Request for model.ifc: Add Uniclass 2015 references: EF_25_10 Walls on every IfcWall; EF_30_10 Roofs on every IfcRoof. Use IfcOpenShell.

First a look at what the model holds.

```python
import ifcopenshell

model = ifcopenshell.open("model.ifc")
print(model.schema)
print("classifications:", [c.Name for c in model.by_type("IfcClassification")])
for ifc_class in ("IfcDoor", "IfcRoof", "IfcStair", "IfcWall", "IfcWindow"):
    print(ifc_class, len(model.by_type(ifc_class)))
```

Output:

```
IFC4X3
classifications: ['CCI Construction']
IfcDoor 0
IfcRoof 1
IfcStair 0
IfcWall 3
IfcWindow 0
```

```python
import ifcopenshell
import ifcopenshell.api.classification

model = ifcopenshell.open("model.ifc")

system = ifcopenshell.api.classification.add_classification(model, classification="Uniclass 2015")

codes = {
    "IfcWall": ("EF_25_10", "Walls"),
    "IfcRoof": ("EF_30_10", "Roofs"),
}
for ifc_class, (code, name) in codes.items():
    products = model.by_type(ifc_class)
    ifcopenshell.api.classification.add_reference(
        model, products=products, classification=system, identification=code, name=name
    )
    print(code, len(products))

model.write("model_v2.ifc")
```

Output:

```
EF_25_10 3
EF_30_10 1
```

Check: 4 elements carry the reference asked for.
